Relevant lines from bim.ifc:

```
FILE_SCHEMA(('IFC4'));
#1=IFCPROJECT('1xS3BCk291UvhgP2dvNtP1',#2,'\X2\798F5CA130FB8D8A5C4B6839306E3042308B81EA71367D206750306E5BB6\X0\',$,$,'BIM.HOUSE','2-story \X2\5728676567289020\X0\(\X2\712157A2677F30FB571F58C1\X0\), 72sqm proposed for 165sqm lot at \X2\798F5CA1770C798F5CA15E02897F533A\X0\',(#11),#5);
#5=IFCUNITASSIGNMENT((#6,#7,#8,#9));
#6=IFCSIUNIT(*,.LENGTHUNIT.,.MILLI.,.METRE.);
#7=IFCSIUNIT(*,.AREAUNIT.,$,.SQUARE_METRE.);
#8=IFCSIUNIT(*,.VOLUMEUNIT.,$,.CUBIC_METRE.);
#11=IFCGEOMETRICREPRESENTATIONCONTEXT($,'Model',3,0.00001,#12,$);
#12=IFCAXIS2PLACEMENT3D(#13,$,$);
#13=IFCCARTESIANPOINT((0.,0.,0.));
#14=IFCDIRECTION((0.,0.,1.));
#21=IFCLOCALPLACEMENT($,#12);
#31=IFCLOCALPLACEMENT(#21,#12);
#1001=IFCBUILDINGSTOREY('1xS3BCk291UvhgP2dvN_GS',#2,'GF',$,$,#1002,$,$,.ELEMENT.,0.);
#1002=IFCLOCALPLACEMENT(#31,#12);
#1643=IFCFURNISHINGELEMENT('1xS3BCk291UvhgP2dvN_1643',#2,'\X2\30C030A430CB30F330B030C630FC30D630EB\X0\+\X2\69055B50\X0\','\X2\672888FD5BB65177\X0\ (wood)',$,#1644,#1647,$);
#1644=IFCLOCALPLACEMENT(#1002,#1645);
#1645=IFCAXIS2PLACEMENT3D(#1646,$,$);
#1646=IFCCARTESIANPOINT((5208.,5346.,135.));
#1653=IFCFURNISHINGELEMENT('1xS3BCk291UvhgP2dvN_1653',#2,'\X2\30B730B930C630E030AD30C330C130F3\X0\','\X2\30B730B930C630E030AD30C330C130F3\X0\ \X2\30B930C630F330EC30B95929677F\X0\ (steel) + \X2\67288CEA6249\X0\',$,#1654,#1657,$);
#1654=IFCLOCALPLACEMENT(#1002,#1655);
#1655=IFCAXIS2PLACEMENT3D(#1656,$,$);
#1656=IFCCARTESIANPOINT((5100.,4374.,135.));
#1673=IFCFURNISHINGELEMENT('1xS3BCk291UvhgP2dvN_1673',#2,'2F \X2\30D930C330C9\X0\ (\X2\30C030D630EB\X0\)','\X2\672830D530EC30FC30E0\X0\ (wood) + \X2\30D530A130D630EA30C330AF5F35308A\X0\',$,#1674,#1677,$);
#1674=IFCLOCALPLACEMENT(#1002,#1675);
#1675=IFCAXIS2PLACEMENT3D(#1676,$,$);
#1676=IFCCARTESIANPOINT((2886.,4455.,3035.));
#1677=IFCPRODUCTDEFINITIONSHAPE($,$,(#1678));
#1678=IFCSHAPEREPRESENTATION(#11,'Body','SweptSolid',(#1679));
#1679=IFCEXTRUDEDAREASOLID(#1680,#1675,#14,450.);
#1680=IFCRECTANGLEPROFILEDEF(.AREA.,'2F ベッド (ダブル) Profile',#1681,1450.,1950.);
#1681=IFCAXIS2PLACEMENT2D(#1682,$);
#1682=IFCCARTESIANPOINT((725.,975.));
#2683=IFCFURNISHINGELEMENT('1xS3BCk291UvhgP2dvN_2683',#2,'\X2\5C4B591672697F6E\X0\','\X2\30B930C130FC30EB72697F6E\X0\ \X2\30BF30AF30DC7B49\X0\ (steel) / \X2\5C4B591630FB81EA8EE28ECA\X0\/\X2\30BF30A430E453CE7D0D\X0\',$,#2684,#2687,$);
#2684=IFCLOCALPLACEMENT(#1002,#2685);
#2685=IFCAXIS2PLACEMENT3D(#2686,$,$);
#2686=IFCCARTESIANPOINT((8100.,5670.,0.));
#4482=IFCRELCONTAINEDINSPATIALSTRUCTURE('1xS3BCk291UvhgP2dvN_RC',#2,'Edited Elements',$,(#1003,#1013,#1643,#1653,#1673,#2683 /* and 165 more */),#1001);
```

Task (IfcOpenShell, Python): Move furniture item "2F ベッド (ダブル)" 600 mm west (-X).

```python
import ifcopenshell
import ifcopenshell.api.geometry
import ifcopenshell.util.placement

model = ifcopenshell.open("bim.ifc")

item = model.by_id(1673)
matrix = ifcopenshell.util.placement.get_local_placement(item.ObjectPlacement)
matrix[0, 3] -= 600.0
ifcopenshell.api.geometry.edit_object_placement(model, product=item, matrix=matrix, is_si=False)

print(ifcopenshell.util.placement.get_local_placement(item.ObjectPlacement).round(3) + 0.0)

model.write("bim_edited.ifc")
```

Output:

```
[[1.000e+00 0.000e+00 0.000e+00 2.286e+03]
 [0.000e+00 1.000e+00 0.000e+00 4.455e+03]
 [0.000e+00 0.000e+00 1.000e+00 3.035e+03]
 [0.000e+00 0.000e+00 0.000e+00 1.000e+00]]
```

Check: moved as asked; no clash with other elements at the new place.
